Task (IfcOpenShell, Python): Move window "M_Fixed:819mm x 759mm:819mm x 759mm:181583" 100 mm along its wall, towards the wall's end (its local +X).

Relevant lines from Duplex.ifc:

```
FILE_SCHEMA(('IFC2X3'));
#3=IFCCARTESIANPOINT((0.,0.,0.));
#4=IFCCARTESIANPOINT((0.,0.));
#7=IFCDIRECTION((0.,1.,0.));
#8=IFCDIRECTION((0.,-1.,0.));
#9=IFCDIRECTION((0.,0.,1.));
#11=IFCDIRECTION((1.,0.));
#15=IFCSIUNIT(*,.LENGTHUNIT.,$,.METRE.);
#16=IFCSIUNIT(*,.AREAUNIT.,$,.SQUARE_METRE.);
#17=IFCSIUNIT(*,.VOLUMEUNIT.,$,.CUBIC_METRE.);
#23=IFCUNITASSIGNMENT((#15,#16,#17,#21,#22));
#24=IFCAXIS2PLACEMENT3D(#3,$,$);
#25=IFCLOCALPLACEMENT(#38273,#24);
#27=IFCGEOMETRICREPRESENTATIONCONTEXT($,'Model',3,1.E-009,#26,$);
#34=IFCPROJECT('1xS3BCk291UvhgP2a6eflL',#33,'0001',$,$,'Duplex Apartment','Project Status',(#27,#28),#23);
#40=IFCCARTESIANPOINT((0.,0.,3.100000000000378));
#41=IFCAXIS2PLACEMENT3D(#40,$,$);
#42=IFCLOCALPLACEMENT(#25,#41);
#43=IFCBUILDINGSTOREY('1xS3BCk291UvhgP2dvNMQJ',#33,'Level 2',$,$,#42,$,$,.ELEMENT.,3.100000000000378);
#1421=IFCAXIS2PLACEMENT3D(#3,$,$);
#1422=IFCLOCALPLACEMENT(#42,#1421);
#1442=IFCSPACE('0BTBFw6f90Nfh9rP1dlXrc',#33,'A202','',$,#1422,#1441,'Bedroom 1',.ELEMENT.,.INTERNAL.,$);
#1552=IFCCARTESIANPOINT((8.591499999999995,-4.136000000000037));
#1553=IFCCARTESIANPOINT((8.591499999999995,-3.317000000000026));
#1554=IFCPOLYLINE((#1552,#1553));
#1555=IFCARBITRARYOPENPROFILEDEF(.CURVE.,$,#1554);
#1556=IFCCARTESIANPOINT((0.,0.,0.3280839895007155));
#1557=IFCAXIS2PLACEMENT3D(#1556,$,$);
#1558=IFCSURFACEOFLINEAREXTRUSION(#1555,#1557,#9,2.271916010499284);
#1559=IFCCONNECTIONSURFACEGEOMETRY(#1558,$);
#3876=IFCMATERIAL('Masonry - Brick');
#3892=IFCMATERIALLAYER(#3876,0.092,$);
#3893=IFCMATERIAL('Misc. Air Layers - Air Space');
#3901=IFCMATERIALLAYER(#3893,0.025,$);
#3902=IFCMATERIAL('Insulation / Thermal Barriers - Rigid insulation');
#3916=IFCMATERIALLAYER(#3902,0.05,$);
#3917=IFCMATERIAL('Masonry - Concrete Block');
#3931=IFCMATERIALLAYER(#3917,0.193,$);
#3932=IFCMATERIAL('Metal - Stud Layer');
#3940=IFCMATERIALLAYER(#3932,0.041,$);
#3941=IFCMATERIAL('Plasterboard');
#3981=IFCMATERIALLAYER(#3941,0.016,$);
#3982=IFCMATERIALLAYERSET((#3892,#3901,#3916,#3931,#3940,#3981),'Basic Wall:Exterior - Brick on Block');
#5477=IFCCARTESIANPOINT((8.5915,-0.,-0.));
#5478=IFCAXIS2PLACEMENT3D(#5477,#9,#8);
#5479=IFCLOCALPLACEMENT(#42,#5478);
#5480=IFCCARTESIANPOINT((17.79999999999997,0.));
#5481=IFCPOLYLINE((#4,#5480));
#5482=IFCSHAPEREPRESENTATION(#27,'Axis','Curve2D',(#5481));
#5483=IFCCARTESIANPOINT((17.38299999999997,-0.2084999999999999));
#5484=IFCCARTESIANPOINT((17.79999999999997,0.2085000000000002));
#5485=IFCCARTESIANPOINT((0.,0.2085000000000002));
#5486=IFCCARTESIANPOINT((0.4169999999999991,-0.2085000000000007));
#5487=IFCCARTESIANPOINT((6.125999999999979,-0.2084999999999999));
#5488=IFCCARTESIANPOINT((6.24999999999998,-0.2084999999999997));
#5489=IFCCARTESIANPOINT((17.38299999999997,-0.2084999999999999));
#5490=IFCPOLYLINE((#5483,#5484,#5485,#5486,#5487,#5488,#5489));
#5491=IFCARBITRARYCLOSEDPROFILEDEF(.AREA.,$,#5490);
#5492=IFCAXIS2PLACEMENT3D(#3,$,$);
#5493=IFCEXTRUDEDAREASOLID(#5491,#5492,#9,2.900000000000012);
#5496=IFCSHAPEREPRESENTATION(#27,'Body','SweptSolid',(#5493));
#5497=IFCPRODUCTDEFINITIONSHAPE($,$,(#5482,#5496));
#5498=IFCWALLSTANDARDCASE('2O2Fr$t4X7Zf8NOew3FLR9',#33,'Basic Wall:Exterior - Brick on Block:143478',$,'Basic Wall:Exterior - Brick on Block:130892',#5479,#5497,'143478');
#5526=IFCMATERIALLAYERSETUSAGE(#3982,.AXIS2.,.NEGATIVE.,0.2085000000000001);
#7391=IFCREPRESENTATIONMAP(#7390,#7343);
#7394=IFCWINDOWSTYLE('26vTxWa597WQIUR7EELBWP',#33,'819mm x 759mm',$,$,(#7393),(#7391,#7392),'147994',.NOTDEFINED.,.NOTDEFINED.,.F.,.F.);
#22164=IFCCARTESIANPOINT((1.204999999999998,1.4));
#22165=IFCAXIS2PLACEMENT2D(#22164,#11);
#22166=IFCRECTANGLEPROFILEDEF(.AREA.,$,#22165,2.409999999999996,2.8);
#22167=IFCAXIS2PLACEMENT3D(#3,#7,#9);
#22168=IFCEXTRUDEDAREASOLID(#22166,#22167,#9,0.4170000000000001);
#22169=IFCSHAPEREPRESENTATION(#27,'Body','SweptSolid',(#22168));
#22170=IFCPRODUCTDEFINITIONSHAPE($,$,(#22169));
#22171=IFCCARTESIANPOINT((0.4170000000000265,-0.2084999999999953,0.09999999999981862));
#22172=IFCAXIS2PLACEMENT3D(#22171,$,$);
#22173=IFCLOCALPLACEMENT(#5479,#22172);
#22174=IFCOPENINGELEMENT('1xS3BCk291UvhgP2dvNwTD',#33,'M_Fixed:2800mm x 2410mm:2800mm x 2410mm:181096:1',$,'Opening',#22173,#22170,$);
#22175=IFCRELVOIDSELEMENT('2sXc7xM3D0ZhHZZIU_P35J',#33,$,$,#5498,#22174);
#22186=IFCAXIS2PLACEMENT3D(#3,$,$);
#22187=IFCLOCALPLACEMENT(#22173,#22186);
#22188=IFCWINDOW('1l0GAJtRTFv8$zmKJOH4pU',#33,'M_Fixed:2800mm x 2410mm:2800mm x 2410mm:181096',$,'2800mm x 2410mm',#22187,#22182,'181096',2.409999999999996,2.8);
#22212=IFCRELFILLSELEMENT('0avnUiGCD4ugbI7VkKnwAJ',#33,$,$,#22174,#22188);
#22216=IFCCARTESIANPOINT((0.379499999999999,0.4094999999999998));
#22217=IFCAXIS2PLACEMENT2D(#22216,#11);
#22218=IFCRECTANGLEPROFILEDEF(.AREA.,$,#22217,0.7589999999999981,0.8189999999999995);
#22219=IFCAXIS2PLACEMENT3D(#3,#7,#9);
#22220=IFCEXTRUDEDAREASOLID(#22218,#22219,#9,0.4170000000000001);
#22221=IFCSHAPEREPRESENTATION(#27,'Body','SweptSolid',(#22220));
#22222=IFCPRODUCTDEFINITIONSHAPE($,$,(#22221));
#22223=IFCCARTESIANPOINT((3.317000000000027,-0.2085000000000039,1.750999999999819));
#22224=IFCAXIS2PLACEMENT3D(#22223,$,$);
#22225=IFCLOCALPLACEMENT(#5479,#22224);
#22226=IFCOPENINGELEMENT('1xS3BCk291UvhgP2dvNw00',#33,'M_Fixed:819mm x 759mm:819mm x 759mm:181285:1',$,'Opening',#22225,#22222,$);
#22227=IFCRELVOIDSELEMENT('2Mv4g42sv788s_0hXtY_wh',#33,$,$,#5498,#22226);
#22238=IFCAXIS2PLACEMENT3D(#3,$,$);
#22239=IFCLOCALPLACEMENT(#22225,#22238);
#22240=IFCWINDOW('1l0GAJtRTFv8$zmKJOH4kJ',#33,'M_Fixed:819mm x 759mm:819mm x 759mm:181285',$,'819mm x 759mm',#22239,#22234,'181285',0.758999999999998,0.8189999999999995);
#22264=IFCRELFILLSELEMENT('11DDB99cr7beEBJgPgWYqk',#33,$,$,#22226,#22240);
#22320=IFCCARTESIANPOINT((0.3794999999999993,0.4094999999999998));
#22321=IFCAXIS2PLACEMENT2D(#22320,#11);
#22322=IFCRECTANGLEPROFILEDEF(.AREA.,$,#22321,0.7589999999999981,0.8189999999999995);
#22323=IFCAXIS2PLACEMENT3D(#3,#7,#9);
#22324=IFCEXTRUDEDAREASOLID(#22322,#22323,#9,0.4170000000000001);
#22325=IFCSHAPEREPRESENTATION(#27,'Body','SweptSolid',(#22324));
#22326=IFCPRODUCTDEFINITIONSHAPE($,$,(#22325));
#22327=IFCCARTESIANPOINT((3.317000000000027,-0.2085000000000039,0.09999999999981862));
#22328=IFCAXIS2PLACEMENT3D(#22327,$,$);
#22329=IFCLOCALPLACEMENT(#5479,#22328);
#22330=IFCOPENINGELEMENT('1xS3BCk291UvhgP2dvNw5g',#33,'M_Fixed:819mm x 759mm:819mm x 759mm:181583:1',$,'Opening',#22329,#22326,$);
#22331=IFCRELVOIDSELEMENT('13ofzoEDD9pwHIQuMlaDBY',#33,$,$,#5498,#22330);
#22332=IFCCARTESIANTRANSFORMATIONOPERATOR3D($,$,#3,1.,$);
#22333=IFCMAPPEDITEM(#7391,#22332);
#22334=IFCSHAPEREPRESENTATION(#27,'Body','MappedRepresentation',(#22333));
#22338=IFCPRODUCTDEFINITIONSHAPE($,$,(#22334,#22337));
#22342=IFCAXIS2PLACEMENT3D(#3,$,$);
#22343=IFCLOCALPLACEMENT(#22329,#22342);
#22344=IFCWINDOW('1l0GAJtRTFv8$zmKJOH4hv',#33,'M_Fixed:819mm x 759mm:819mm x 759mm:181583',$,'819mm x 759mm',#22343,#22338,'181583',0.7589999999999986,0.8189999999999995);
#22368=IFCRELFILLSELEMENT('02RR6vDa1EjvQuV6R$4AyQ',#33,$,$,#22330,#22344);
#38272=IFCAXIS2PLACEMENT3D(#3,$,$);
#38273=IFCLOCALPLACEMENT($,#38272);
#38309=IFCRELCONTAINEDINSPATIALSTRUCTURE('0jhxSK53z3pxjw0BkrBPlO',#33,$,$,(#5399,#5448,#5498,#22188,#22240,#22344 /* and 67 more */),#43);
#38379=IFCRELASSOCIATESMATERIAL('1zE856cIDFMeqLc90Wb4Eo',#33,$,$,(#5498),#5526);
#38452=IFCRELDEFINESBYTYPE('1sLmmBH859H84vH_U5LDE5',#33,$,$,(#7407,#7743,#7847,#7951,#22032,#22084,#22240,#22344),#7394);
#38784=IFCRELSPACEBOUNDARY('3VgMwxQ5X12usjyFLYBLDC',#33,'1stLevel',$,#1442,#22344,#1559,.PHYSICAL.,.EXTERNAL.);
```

```python
import numpy as np
import ifcopenshell
import ifcopenshell.api.geometry
import ifcopenshell.util.placement

model = ifcopenshell.open("Duplex.ifc")

window = model.by_id(22344)
opening = window.FillsVoids[0].RelatingOpeningElement
wall = opening.VoidsElements[0].RelatingBuildingElement

wall_matrix = ifcopenshell.util.placement.get_local_placement(wall.ObjectPlacement)
shift = wall_matrix[:3, 0] * 0.1
before = ifcopenshell.util.placement.get_local_placement(window.ObjectPlacement)[:3, 3].copy()

# The window is placed relative to its opening, so it follows when the opening moves.
matrix = ifcopenshell.util.placement.get_local_placement(opening.ObjectPlacement)
matrix[:3, 3] += shift
ifcopenshell.api.geometry.edit_object_placement(
    model, product=opening, matrix=matrix, is_si=False, should_transform_children=True
)

# Space boundary surfaces are stored in each space's coordinates; move them too.
for rel in window.ProvidesBoundaries:
    if not rel.ConnectionGeometry:
        continue
    surface = rel.ConnectionGeometry.SurfaceOnRelatingElement
    space_matrix = ifcopenshell.util.placement.get_local_placement(rel.RelatingSpace.ObjectPlacement)
    point = np.array(surface.Position.Location.Coordinates) + space_matrix[:3, :3].T @ shift
    surface.Position = model.createIfcAxis2Placement3D(
        model.createIfcCartesianPoint(point.tolist()), surface.Position.Axis, surface.Position.RefDirection
    )

after = ifcopenshell.util.placement.get_local_placement(window.ObjectPlacement)[:3, 3]
print("window moved by", (after - before).round(3) + 0.0)

model.write("Duplex_v2.ifc")
```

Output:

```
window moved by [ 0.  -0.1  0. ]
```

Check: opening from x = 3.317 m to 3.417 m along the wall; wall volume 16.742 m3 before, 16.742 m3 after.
